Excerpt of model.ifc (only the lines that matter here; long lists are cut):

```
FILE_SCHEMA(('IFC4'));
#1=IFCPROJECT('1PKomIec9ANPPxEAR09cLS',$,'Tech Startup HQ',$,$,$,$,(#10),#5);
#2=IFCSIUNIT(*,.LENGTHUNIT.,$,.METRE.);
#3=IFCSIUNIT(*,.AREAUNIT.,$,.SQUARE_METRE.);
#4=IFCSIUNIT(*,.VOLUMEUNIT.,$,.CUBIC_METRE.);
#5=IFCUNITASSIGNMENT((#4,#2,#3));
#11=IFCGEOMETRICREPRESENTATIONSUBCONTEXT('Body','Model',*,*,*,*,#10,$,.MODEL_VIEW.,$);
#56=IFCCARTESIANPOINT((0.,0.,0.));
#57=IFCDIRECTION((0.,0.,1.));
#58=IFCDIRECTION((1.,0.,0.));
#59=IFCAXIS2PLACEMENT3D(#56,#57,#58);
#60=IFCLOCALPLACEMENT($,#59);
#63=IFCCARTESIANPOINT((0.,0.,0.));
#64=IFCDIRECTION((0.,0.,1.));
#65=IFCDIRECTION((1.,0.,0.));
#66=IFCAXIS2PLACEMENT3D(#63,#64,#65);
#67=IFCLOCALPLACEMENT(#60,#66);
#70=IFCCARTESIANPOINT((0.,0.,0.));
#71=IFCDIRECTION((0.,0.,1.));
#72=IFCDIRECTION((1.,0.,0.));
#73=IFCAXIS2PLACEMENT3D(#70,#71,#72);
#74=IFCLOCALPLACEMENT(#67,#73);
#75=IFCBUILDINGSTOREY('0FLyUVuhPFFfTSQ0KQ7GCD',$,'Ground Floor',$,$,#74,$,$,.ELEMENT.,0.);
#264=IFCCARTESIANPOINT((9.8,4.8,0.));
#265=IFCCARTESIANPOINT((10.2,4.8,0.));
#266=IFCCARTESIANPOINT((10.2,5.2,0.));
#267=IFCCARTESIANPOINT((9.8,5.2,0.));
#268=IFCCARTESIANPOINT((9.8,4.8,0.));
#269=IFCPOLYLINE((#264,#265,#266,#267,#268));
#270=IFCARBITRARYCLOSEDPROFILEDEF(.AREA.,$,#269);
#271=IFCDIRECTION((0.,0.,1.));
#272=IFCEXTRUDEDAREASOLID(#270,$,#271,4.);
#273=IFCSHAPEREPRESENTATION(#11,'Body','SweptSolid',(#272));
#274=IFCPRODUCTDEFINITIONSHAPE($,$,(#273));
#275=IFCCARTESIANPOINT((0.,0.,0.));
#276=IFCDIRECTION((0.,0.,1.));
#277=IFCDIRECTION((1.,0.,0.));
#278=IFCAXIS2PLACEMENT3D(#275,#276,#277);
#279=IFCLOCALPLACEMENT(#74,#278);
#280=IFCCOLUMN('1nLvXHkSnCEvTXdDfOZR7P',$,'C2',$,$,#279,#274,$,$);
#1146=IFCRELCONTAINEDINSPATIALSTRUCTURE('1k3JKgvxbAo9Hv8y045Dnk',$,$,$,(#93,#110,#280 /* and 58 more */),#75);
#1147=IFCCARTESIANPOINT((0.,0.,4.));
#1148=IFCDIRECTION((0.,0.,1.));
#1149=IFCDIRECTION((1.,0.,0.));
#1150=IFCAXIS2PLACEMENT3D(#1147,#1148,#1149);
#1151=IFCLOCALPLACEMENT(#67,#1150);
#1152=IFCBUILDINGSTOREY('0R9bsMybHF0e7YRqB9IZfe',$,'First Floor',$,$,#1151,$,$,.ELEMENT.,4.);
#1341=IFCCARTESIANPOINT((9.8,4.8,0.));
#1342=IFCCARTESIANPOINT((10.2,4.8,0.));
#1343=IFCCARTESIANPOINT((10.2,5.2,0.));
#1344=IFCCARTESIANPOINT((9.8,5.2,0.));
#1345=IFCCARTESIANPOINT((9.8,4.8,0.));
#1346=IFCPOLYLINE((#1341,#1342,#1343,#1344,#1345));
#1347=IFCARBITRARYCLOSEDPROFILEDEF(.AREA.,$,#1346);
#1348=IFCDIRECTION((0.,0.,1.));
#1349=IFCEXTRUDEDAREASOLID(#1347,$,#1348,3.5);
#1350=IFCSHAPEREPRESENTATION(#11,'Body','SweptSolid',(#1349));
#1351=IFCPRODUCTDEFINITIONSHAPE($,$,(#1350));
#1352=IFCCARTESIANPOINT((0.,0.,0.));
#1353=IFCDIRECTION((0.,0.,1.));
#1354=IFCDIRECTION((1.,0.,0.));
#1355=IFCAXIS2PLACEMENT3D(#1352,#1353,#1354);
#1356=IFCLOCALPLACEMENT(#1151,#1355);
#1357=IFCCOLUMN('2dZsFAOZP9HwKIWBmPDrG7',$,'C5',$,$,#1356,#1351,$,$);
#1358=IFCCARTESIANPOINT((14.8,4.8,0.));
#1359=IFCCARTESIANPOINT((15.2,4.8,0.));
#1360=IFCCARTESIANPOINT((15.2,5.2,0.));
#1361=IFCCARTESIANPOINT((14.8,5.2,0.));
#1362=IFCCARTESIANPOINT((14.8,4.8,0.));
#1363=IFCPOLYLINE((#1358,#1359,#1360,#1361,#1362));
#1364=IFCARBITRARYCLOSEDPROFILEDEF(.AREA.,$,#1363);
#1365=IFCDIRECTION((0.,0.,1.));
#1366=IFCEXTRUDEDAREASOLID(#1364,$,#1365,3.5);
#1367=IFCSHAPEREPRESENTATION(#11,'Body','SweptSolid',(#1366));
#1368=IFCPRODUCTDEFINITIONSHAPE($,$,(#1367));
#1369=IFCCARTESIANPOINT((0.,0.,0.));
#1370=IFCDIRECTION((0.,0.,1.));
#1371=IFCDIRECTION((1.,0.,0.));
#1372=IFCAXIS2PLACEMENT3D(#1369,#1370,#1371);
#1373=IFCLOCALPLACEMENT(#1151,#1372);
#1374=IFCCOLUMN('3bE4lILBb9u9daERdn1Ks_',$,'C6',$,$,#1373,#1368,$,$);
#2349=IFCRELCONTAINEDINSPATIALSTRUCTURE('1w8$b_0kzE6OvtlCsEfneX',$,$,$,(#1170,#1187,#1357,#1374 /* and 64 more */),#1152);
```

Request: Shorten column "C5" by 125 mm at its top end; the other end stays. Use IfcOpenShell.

```python
import ifcopenshell
import ifcopenshell.util.representation
import ifcopenshell.util.unit

model = ifcopenshell.open("model.ifc")
unit_scale = ifcopenshell.util.unit.calculate_unit_scale(model)

member = model.by_guid("2dZsFAOZP9HwKIWBmPDrG7")
change = -0.125 / unit_scale

# The extrusion runs towards the end named, so only its depth changes.
body = ifcopenshell.util.representation.get_representation(member, "Model", "Body")
solid = body.Items[0]
old_length = solid.Depth
solid.Depth += change

print(f"length {old_length:g} -> {solid.Depth:g}")

model.write("model_updated.ifc")
```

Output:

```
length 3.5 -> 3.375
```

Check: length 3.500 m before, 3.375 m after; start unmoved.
